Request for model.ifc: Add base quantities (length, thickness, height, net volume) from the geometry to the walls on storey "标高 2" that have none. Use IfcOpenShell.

First a look at what the model holds.

```python
import ifcopenshell
import ifcopenshell.util.element
import ifcopenshell.util.unit

model = ifcopenshell.open("model.ifc")
print(model.schema)
for unit_type in ("LENGTHUNIT", "AREAUNIT", "VOLUMEUNIT"):
    print(unit_type, ifcopenshell.util.unit.calculate_unit_scale(model, unit_type))
storey = next(s for s in model.by_type("IfcBuildingStorey") if s.Name == "标高 2")
walls = [e for e in ifcopenshell.util.element.get_decomposition(storey) if e.is_a("IfcWall")]
for e in sorted(walls, key=lambda e: e.id()):
    print(e.id(), e.is_a(), e.Name, list(ifcopenshell.util.element.get_psets(e, qtos_only=True)), sep=" | ")
```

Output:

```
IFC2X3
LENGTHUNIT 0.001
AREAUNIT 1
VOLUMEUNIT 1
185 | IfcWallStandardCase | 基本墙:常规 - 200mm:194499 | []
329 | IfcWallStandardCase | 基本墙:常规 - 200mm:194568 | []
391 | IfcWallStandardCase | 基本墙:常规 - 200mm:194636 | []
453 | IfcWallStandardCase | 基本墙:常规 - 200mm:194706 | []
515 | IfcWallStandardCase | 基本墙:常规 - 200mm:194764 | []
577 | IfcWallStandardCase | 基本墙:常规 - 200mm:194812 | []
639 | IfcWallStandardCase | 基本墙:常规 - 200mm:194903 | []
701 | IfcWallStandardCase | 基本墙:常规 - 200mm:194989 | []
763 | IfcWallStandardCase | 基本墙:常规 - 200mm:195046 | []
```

```python
import ifcopenshell
import ifcopenshell.api.pset
import ifcopenshell.geom
import ifcopenshell.util.element
import ifcopenshell.util.shape
import ifcopenshell.util.unit

model = ifcopenshell.open("model.ifc")
unit_scale = ifcopenshell.util.unit.calculate_unit_scale(model)
volume_scale = ifcopenshell.util.unit.calculate_unit_scale(model, "VOLUMEUNIT")
settings = ifcopenshell.geom.settings()

storey = next(s for s in model.by_type("IfcBuildingStorey") if s.Name == "标高 2")
walls = [e for e in ifcopenshell.util.element.get_decomposition(storey) if e.is_a("IfcWall")]

for e in sorted(walls, key=lambda e: e.id()):
    if ifcopenshell.util.element.get_psets(e, qtos_only=True, should_inherit=False):
        continue
    # Geometry comes back in metres, in the element's own axes.
    shape = ifcopenshell.geom.create_shape(settings, e)
    values = {
        "Length": ifcopenshell.util.shape.get_x(shape.geometry) / unit_scale,
        "Width": ifcopenshell.util.shape.get_y(shape.geometry) / unit_scale,
        "Height": ifcopenshell.util.shape.get_z(shape.geometry) / unit_scale,
        "NetVolume": ifcopenshell.util.shape.get_volume(shape.geometry) / volume_scale,
    }
    qto = ifcopenshell.api.pset.add_qto(model, product=e, name="BaseQuantities")
    ifcopenshell.api.pset.edit_qto(model, qto=qto, properties=values)
    print(e.id(), {k: round(v, 3) for k, v in values.items()})

model.write("model_updated.ifc")
```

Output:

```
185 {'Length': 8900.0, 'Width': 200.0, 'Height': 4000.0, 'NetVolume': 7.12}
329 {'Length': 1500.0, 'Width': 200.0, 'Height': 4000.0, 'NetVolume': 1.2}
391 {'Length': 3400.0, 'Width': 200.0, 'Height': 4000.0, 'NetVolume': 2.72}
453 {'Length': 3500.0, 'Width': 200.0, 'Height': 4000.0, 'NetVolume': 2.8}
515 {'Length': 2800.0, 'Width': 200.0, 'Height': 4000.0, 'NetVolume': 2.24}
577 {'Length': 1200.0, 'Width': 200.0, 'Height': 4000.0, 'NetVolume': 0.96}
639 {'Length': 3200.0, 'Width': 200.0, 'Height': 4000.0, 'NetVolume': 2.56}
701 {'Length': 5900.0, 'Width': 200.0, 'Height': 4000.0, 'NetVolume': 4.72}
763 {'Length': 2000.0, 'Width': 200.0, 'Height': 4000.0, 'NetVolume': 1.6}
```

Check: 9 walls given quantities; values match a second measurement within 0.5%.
